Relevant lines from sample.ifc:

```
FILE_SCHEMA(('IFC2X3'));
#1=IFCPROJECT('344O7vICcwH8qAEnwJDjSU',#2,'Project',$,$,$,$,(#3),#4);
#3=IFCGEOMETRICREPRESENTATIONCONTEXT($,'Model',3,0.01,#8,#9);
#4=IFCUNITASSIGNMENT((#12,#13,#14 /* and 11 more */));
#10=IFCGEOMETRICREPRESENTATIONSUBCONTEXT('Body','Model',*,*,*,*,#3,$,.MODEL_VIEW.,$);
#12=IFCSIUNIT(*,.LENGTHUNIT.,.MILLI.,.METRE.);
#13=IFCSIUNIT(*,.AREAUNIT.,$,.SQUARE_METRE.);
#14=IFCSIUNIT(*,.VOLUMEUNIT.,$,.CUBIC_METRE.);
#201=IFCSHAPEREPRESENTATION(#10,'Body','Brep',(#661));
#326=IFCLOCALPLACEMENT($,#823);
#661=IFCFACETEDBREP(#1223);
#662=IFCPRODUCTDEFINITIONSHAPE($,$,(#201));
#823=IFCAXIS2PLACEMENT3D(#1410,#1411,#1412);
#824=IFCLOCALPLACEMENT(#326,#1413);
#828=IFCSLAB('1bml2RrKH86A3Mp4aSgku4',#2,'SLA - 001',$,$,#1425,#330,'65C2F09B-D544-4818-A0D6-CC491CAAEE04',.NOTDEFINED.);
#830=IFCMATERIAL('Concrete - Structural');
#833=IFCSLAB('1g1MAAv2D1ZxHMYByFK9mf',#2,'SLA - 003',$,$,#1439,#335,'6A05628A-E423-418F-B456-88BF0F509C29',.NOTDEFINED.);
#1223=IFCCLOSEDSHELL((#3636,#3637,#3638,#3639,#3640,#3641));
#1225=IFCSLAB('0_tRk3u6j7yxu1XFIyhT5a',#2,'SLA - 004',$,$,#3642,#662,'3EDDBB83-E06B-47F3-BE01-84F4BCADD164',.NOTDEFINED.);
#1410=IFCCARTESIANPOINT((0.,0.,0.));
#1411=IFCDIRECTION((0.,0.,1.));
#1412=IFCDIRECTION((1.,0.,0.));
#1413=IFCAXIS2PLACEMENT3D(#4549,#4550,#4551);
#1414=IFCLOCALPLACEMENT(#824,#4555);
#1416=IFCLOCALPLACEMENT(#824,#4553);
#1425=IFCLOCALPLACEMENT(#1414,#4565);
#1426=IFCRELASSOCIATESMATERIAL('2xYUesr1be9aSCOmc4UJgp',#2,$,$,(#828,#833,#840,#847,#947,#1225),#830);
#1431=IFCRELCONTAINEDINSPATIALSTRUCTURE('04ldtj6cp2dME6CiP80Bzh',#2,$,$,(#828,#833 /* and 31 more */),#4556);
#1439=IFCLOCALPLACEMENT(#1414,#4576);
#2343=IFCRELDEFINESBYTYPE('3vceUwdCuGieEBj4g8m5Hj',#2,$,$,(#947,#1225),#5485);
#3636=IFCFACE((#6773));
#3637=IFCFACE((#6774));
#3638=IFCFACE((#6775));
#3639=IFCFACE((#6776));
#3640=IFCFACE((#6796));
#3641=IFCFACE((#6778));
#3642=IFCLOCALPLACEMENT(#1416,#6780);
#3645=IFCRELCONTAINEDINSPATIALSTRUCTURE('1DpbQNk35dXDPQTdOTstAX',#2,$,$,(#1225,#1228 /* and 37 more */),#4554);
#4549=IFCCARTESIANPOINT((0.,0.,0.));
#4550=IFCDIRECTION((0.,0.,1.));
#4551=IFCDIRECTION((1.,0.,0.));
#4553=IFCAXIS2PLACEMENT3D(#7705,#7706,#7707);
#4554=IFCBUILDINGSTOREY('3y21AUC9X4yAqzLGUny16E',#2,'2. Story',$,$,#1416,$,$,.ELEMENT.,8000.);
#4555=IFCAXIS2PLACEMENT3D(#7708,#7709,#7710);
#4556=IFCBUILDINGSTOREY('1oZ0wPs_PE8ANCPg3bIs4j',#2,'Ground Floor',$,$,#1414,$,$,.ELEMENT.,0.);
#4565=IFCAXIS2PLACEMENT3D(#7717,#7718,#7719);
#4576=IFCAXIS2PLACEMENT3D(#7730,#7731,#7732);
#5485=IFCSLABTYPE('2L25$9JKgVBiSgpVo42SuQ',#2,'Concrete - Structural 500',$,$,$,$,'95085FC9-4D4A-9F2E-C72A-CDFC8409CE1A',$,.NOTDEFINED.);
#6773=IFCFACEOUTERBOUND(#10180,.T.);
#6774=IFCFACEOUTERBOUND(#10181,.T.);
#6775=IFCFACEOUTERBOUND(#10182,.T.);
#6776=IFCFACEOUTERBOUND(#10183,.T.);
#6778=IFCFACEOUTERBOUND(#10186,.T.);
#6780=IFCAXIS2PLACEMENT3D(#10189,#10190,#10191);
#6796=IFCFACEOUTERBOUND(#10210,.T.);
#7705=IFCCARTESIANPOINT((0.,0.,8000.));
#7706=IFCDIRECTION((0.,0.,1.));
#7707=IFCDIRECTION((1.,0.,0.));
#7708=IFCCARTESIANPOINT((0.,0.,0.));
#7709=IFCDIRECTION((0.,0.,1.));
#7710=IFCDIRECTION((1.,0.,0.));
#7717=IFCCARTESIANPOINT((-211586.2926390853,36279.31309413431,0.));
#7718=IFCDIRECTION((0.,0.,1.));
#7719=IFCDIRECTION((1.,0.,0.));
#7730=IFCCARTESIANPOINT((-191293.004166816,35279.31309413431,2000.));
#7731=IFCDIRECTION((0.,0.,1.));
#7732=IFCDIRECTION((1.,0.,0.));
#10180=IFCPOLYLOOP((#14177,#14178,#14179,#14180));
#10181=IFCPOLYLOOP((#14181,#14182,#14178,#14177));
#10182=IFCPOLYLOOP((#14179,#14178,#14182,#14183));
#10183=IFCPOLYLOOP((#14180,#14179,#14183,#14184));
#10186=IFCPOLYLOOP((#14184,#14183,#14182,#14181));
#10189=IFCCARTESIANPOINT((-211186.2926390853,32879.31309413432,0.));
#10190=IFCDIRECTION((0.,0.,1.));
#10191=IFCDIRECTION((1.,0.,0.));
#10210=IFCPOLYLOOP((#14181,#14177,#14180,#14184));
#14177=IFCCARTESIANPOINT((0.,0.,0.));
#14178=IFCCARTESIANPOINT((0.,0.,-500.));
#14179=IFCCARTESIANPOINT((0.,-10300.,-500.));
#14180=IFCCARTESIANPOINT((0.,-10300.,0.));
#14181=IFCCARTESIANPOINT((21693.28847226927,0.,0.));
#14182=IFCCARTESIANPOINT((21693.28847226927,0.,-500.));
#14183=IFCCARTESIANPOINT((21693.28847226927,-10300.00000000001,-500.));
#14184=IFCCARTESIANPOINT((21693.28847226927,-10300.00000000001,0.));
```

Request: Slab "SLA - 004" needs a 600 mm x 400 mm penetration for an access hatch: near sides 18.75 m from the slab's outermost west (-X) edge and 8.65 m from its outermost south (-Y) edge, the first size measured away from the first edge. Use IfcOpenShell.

```python
import numpy as np
import ifcopenshell
import ifcopenshell.api.feature
import ifcopenshell.api.geometry
import ifcopenshell.api.root
import ifcopenshell.geom
import ifcopenshell.util.placement
import ifcopenshell.util.representation
import ifcopenshell.util.shape
import ifcopenshell.util.unit

model = ifcopenshell.open("sample.ifc")
unit_scale = ifcopenshell.util.unit.calculate_unit_scale(model)
settings = ifcopenshell.geom.settings()


def volume(element):
    """Net volume in cubic metres, openings subtracted."""
    shape = ifcopenshell.geom.create_shape(settings, element)
    return ifcopenshell.util.shape.get_volume(shape.geometry)


slab = model.by_guid("0_tRk3u6j7yxu1XFIyhT5a")
before = volume(slab)

# Extent in the slab's own axes, in metres. The edges named are its -X and -Y sides.
slab_shape = ifcopenshell.geom.create_shape(settings, slab)
vertices = ifcopenshell.util.shape.get_vertices(slab_shape.geometry)
x_min, y_min, bottom = vertices.min(axis=0)
top = vertices[:, 2].max()

opening = ifcopenshell.api.root.create_entity(model, ifc_class="IfcOpeningElement", name="Access hatch opening")
context = ifcopenshell.util.representation.get_context(model, "Model", "Body", "MODEL_VIEW")
width, depth = 0.6, 0.4
outline = [(0.0, 0.0), (width, 0.0), (width, depth), (0.0, depth), (0.0, 0.0)]
# Overshoot both faces by 50 mm so the cut is clean.
shape = ifcopenshell.api.geometry.add_slab_representation(
    model, context=context, depth=top - bottom + 0.1, polyline=outline
)
ifcopenshell.api.geometry.assign_representation(model, product=opening, representation=shape)

matrix = ifcopenshell.util.placement.get_local_placement(slab.ObjectPlacement)
matrix[:, 3] = matrix @ np.append(np.array([x_min + 18.75, y_min + 8.65, bottom - 0.05]) / unit_scale, 1.0)
ifcopenshell.api.geometry.edit_object_placement(model, product=opening, matrix=matrix, is_si=False)
ifcopenshell.api.feature.add_feature(model, feature=opening, element=slab)

after = volume(slab)

print(f"slab volume {before:.3f} -> {after:.3f} m3")

model.write("sample_rev.ifc")
```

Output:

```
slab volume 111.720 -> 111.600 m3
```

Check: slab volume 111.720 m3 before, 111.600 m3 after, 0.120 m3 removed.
